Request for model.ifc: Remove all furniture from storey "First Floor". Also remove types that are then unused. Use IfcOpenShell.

First a look at what the model holds.

```python
import ifcopenshell
import ifcopenshell.util.element

model = ifcopenshell.open("model.ifc")
print(model.schema)
storey = next(s for s in model.by_type("IfcBuildingStorey") if s.Name == "First Floor")
furniture = [e for e in ifcopenshell.util.element.get_decomposition(storey) if e.is_a("IfcFurnishingElement")]
seen = {}
for e in furniture:
    element_type = ifcopenshell.util.element.get_type(e)
    name = element_type.Name if element_type not in (None, e) else None
    seen[name] = seen.get(name, 0) + 1
for name, count in sorted(seen.items(), key=str):
    print(count, "x", name)
```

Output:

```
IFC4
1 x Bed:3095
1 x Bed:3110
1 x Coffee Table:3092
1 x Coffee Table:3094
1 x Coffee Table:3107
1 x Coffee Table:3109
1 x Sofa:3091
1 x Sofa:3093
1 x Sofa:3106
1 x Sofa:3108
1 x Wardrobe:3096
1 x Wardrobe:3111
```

```python
import ifcopenshell
import ifcopenshell.api.root
import ifcopenshell.util.element

model = ifcopenshell.open("model.ifc")

storey = next(s for s in model.by_type("IfcBuildingStorey") if s.Name == "First Floor")
furniture = [e for e in ifcopenshell.util.element.get_decomposition(storey) if e.is_a("IfcFurnishingElement")]
types = {ifcopenshell.util.element.get_type(e) for e in furniture} - {None, *furniture}

for e in furniture:
    ifcopenshell.api.root.remove_product(model, product=e)
print(len(furniture), "removed")

unused = [t for t in types if not ifcopenshell.util.element.get_types(t)]
for t in unused:
    ifcopenshell.api.root.remove_product(model, product=t)
print(len(unused), "unused types removed")

model.write("model_edited.ifc")
```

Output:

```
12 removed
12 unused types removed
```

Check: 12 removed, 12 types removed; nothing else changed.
